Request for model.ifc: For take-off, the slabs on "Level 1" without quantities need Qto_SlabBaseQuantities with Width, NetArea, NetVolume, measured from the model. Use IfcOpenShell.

First a look at what the model holds.

```python
import ifcopenshell
import ifcopenshell.util.element
import ifcopenshell.util.unit

model = ifcopenshell.open("model.ifc")
print(model.schema)
for unit_type in ("LENGTHUNIT", "AREAUNIT", "VOLUMEUNIT"):
    print(unit_type, ifcopenshell.util.unit.calculate_unit_scale(model, unit_type))
storey = next(s for s in model.by_type("IfcBuildingStorey") if s.Name == "Level 1")
slabs = [e for e in ifcopenshell.util.element.get_decomposition(storey) if e.is_a("IfcSlab")]
for e in sorted(slabs, key=lambda e: e.id()):
    print(e.id(), e.is_a(), e.Name, list(ifcopenshell.util.element.get_psets(e, qtos_only=True)), sep=" | ")
```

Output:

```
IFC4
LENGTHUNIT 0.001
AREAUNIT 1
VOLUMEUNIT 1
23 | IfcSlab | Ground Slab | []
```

```python
import ifcopenshell
import ifcopenshell.api.pset
import ifcopenshell.geom
import ifcopenshell.util.element
import ifcopenshell.util.shape
import ifcopenshell.util.unit

model = ifcopenshell.open("model.ifc")
unit_scale = ifcopenshell.util.unit.calculate_unit_scale(model)
area_scale = ifcopenshell.util.unit.calculate_unit_scale(model, "AREAUNIT")
volume_scale = ifcopenshell.util.unit.calculate_unit_scale(model, "VOLUMEUNIT")
settings = ifcopenshell.geom.settings()

storey = next(s for s in model.by_type("IfcBuildingStorey") if s.Name == "Level 1")
slabs = [e for e in ifcopenshell.util.element.get_decomposition(storey) if e.is_a("IfcSlab")]

for e in sorted(slabs, key=lambda e: e.id()):
    if ifcopenshell.util.element.get_psets(e, qtos_only=True, should_inherit=False):
        continue
    # Geometry comes back in metres, in the element's own axes.
    shape = ifcopenshell.geom.create_shape(settings, e)
    values = {
        "Width": ifcopenshell.util.shape.get_z(shape.geometry) / unit_scale,
        "NetArea": ifcopenshell.util.shape.get_footprint_area(shape.geometry) / area_scale,
        "NetVolume": ifcopenshell.util.shape.get_volume(shape.geometry) / volume_scale,
    }
    qto = ifcopenshell.api.pset.add_qto(model, product=e, name="Qto_SlabBaseQuantities")
    ifcopenshell.api.pset.edit_qto(model, qto=qto, properties=values)
    print(e.id(), {k: round(v, 3) for k, v in values.items()})

model.write("model_updated.ifc")
```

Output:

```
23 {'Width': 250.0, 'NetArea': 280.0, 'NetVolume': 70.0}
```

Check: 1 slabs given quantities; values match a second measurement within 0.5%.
